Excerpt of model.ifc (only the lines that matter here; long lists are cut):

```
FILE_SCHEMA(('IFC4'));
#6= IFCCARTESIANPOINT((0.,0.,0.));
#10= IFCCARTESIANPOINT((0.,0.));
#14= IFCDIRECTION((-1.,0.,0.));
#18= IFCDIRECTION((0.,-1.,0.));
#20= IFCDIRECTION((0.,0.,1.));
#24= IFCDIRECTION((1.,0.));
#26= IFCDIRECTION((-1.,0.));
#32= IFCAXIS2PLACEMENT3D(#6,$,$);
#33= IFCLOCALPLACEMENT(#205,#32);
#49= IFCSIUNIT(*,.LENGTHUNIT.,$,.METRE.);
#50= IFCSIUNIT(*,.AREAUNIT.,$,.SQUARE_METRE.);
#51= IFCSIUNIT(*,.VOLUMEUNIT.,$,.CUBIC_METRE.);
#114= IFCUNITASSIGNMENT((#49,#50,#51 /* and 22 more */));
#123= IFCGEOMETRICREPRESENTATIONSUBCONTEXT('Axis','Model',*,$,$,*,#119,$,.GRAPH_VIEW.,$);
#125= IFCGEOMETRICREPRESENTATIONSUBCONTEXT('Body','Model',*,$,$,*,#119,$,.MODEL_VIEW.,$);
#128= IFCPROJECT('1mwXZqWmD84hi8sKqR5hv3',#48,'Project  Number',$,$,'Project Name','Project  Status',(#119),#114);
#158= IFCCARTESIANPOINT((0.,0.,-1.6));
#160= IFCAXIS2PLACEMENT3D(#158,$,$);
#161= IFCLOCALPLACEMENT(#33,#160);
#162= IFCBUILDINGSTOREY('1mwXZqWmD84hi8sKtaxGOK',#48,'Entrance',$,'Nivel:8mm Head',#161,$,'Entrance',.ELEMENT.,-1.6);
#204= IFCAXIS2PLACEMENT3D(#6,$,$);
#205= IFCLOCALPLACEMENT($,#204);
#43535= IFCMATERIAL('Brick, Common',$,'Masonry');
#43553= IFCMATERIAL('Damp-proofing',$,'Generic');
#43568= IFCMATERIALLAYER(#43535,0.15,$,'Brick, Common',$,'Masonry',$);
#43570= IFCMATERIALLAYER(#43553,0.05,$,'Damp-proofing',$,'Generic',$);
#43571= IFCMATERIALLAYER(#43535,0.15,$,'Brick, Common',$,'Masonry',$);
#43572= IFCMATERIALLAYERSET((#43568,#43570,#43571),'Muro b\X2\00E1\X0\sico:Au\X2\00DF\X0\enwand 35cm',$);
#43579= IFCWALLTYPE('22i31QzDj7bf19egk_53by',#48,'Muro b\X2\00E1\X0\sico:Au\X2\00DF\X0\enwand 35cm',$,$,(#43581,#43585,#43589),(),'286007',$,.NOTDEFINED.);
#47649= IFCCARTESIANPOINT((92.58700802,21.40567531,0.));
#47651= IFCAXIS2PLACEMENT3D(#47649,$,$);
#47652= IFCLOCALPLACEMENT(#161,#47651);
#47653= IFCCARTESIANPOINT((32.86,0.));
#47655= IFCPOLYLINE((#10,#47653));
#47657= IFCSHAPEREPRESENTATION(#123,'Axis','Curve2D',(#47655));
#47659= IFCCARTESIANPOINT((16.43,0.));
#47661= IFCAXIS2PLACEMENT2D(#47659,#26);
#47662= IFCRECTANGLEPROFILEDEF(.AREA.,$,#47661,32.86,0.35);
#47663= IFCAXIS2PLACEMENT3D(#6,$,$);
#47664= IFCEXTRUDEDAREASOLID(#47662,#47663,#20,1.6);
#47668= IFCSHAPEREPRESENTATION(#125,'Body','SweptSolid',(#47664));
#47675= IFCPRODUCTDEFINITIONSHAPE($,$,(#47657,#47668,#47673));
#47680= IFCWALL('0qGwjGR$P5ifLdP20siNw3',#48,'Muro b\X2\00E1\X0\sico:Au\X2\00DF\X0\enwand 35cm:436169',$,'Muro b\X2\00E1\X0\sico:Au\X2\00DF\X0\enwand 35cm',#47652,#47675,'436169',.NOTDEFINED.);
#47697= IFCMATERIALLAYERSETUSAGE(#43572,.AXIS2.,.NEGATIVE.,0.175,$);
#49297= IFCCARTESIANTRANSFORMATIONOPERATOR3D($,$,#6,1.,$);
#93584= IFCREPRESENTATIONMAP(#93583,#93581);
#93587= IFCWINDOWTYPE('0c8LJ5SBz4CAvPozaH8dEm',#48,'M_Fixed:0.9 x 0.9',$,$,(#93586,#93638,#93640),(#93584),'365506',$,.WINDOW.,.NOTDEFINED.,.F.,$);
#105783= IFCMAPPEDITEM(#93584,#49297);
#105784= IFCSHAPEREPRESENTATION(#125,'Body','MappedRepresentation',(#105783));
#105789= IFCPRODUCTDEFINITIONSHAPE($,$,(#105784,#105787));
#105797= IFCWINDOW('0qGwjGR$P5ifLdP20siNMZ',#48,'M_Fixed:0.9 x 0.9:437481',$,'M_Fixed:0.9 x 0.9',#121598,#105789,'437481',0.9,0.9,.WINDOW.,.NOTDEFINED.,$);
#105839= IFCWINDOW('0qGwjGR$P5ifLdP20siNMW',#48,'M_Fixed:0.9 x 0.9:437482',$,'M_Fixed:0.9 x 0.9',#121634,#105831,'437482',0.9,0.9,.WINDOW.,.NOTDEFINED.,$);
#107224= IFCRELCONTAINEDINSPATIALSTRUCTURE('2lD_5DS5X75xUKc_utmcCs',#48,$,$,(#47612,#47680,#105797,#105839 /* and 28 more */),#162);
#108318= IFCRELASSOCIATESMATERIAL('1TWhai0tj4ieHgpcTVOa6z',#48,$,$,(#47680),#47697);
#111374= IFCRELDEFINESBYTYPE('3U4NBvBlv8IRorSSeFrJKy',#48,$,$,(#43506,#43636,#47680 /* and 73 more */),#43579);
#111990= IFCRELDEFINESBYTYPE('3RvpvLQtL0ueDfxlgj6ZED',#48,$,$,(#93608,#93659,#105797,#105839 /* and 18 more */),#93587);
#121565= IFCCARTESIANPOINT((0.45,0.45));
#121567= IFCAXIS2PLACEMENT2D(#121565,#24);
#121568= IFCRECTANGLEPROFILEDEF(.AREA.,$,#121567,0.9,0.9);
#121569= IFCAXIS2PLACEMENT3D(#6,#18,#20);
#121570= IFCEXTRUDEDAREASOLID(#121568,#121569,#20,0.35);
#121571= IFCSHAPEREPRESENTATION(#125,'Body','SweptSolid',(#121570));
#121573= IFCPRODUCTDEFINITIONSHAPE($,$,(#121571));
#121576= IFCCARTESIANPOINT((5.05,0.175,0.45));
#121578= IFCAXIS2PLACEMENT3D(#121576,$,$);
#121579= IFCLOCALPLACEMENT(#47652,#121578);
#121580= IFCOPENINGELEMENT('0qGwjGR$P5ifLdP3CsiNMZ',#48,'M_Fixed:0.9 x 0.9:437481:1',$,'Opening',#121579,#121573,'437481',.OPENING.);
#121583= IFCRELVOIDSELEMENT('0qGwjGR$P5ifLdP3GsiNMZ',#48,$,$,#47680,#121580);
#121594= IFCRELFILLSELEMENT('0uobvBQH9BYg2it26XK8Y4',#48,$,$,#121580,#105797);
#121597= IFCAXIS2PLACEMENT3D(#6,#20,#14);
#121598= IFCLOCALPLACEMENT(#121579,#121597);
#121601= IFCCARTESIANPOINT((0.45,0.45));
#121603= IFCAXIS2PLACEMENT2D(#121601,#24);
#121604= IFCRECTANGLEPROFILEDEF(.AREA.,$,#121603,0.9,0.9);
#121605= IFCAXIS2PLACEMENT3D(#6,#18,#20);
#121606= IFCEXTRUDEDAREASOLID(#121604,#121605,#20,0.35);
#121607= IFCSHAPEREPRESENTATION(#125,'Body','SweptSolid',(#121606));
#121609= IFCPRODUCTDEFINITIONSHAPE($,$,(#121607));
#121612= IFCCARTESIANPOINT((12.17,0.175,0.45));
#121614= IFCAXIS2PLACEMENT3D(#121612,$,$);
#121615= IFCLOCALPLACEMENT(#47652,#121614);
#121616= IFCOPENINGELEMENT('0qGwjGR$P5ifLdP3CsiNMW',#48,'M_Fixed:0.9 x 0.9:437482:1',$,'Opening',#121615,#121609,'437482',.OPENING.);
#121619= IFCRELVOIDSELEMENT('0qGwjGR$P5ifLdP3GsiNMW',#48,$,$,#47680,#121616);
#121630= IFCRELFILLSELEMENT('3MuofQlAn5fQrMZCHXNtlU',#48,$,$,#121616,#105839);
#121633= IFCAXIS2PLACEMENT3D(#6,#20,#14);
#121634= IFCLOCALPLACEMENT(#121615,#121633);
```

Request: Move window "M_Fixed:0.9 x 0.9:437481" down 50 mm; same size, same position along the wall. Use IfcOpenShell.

```python
import numpy as np
import ifcopenshell
import ifcopenshell.api.geometry
import ifcopenshell.util.placement
import ifcopenshell.util.unit

model = ifcopenshell.open("model.ifc")
unit_scale = ifcopenshell.util.unit.calculate_unit_scale(model)

window = model.by_guid("0qGwjGR$P5ifLdP20siNMZ")
opening = window.FillsVoids[0].RelatingOpeningElement
dz = -0.05 / unit_scale

shift = np.array([0.0, 0.0, dz])
# The window is placed relative to its opening, so it follows when the opening moves.
matrix = ifcopenshell.util.placement.get_local_placement(opening.ObjectPlacement)
matrix[:3, 3] += shift
ifcopenshell.api.geometry.edit_object_placement(
    model, product=opening, matrix=matrix, is_si=False, should_transform_children=True
)

print(f"moved by {dz * unit_scale:+.3f} m")

model.write("model_rev.ifc")
```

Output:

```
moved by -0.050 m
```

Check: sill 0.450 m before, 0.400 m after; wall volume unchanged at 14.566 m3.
